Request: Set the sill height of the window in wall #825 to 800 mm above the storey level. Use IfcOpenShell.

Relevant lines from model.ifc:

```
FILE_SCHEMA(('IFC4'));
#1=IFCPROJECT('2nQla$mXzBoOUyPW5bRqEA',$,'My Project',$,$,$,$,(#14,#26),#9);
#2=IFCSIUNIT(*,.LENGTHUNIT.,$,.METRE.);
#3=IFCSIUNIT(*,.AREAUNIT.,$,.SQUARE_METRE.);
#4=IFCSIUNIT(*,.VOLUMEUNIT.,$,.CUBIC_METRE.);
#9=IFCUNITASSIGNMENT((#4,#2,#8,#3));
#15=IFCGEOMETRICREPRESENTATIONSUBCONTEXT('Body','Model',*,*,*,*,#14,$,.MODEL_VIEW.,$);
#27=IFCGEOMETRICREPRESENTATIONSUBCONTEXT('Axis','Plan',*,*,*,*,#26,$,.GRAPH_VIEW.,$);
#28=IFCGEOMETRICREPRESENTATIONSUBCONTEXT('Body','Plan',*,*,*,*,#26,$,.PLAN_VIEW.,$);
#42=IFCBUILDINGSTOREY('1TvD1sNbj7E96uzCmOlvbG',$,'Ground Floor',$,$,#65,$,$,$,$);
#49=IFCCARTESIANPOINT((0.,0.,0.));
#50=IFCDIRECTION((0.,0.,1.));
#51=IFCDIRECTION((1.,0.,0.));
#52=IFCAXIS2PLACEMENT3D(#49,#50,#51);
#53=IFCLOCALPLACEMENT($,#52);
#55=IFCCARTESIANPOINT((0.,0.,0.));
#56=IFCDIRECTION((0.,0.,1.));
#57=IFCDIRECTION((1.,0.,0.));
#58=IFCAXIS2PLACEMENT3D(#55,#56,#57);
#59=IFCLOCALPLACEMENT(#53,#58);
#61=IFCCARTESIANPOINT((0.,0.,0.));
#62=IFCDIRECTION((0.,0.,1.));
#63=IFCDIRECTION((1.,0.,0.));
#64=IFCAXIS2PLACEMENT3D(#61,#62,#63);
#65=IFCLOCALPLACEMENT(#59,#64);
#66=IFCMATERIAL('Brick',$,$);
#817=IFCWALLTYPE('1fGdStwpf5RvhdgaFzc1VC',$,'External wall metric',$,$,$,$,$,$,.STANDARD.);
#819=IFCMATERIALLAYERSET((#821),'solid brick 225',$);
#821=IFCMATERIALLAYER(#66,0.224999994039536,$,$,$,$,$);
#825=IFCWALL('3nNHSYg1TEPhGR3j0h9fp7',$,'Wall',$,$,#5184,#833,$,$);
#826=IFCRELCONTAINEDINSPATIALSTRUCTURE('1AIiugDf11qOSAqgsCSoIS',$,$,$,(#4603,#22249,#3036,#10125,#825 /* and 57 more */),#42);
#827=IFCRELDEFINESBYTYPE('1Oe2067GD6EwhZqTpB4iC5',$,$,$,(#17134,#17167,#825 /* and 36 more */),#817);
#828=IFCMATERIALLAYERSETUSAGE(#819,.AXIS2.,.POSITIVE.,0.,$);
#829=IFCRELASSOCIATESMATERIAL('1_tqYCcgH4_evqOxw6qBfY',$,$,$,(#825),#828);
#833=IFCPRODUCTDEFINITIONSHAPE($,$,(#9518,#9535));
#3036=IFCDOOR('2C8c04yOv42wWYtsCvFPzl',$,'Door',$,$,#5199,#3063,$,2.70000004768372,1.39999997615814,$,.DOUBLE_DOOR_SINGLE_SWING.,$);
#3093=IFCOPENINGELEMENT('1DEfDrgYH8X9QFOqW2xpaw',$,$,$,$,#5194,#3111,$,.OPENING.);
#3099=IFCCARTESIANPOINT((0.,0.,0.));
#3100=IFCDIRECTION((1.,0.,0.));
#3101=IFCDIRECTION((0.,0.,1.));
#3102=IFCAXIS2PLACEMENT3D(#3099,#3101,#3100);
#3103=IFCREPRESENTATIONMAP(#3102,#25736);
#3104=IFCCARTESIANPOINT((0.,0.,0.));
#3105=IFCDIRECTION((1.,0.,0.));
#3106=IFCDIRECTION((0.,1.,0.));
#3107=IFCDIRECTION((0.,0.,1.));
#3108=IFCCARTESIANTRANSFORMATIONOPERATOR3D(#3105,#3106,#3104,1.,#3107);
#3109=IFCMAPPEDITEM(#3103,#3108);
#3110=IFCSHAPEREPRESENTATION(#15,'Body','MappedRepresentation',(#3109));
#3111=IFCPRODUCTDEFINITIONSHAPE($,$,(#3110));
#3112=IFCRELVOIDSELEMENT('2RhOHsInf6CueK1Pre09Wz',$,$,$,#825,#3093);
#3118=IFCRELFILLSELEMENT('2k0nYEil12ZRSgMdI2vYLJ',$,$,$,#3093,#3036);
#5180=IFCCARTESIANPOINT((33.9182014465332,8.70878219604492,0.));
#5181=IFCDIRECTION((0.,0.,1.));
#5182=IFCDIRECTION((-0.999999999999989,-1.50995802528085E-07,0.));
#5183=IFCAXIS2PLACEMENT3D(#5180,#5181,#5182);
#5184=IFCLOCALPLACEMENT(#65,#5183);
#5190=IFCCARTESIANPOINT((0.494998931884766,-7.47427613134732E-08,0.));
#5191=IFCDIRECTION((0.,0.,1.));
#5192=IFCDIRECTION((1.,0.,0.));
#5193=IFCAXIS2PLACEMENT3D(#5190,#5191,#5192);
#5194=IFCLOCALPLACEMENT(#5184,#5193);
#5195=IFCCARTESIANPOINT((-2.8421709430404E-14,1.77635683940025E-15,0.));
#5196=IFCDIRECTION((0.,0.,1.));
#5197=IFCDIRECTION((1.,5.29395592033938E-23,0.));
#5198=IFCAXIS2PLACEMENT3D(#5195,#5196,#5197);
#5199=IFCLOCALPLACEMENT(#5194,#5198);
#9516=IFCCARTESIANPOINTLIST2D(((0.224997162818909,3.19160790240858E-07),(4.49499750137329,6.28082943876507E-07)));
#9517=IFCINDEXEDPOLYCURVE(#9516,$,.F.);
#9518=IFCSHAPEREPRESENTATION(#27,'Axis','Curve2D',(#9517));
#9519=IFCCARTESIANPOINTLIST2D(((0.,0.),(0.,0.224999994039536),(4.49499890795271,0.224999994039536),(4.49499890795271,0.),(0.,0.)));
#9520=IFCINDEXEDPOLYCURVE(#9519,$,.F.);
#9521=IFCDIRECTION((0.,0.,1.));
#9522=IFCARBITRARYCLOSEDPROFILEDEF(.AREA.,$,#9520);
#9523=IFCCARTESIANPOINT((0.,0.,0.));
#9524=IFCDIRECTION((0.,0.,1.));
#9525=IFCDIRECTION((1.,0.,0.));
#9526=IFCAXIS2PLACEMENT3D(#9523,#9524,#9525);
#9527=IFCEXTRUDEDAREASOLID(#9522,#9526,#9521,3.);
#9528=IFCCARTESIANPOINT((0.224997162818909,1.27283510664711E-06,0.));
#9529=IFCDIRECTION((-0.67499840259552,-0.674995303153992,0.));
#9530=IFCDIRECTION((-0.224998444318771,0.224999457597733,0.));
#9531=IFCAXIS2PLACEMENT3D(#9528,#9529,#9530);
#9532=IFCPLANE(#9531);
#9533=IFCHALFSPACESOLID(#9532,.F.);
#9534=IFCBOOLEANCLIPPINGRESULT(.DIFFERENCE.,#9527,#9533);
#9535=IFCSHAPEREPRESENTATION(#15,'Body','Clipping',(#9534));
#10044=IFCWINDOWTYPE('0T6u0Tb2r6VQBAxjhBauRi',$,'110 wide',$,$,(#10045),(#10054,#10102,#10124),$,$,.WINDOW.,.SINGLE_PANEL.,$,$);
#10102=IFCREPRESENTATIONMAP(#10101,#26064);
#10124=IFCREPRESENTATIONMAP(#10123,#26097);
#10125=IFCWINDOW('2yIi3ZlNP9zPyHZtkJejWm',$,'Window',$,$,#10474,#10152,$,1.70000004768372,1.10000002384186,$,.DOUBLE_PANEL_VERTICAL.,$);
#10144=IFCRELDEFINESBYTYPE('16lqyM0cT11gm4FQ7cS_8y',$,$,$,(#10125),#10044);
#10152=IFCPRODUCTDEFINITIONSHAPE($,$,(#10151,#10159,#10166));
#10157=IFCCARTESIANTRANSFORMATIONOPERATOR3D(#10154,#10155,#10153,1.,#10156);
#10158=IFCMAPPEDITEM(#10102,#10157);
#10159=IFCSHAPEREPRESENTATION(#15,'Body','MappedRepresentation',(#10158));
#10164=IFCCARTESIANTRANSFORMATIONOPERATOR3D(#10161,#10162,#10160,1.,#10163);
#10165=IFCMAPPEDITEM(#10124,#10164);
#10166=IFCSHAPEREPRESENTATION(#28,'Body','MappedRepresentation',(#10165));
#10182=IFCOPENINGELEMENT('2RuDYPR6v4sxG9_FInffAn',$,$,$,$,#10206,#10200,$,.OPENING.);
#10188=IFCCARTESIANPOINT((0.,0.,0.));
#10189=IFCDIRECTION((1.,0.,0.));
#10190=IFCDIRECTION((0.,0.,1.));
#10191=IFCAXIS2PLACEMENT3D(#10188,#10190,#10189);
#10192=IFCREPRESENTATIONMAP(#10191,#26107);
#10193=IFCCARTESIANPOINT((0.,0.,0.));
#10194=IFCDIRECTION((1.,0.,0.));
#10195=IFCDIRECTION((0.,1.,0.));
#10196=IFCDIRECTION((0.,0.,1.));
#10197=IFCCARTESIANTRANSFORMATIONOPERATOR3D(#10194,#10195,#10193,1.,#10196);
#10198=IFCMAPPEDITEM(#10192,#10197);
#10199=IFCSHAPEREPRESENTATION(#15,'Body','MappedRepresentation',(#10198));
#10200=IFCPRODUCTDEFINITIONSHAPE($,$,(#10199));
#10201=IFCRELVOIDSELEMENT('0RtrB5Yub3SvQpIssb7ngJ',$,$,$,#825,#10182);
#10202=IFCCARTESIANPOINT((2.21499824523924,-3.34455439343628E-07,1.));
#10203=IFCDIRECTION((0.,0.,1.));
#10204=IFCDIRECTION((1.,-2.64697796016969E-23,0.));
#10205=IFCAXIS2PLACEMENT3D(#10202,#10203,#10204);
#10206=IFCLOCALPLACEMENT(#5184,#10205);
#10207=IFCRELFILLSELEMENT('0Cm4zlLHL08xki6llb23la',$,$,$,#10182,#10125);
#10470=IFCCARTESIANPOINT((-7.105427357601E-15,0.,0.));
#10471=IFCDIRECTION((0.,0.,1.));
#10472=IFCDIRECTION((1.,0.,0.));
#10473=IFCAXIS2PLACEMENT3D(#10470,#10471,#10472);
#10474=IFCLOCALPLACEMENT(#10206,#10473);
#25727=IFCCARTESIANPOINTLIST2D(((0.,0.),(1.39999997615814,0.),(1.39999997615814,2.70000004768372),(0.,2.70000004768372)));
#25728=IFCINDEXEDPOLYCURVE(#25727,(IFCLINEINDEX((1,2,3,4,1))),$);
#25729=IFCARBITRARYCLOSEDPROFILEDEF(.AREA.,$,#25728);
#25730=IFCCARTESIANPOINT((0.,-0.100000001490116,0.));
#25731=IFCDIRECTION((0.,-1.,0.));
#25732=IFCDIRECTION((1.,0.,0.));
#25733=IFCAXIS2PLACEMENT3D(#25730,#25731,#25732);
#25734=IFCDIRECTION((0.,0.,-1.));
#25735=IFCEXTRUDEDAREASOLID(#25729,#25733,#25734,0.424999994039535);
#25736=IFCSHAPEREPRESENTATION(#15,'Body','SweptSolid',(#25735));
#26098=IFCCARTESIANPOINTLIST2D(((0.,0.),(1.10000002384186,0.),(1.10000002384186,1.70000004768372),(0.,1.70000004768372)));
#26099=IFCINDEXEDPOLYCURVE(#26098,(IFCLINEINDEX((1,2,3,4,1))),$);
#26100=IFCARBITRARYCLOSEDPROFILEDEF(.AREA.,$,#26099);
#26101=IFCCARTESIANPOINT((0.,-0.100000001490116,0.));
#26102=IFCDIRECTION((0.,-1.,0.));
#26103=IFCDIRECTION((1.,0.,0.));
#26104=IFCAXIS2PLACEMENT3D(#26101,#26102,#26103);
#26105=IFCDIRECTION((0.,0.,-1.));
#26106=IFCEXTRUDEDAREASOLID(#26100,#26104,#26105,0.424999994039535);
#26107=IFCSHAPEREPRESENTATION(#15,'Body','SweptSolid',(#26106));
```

```python
import numpy as np
import ifcopenshell
import ifcopenshell.api.geometry
import ifcopenshell.geom
import ifcopenshell.util.element
import ifcopenshell.util.placement
import ifcopenshell.util.shape
import ifcopenshell.util.unit

model = ifcopenshell.open("model.ifc")
unit_scale = ifcopenshell.util.unit.calculate_unit_scale(model)

window = model.by_guid("2yIi3ZlNP9zPyHZtkJejWm")
opening = window.FillsVoids[0].RelatingOpeningElement
storey = ifcopenshell.util.element.get_container(window, ifc_class="IfcBuildingStorey")
level = ifcopenshell.util.placement.get_local_placement(storey.ObjectPlacement)[2, 3]

# The opening's origin need not be at the sill, so measure its lowest point.
shape = ifcopenshell.geom.create_shape(ifcopenshell.geom.settings(), opening)
bottom = ifcopenshell.util.shape.get_shape_bottom_elevation(shape, shape.geometry) / unit_scale
dz = level + 0.8 - bottom

shift = np.array([0.0, 0.0, dz])
# The window is placed relative to its opening, so it follows when the opening moves.
matrix = ifcopenshell.util.placement.get_local_placement(opening.ObjectPlacement)
matrix[:3, 3] += shift
ifcopenshell.api.geometry.edit_object_placement(
    model, product=opening, matrix=matrix, is_si=False, should_transform_children=True
)

print(f"moved by {dz * unit_scale:+.3f} m")

model.write("model_edited.ifc")
```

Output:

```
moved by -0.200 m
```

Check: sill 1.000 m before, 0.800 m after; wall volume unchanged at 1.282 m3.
